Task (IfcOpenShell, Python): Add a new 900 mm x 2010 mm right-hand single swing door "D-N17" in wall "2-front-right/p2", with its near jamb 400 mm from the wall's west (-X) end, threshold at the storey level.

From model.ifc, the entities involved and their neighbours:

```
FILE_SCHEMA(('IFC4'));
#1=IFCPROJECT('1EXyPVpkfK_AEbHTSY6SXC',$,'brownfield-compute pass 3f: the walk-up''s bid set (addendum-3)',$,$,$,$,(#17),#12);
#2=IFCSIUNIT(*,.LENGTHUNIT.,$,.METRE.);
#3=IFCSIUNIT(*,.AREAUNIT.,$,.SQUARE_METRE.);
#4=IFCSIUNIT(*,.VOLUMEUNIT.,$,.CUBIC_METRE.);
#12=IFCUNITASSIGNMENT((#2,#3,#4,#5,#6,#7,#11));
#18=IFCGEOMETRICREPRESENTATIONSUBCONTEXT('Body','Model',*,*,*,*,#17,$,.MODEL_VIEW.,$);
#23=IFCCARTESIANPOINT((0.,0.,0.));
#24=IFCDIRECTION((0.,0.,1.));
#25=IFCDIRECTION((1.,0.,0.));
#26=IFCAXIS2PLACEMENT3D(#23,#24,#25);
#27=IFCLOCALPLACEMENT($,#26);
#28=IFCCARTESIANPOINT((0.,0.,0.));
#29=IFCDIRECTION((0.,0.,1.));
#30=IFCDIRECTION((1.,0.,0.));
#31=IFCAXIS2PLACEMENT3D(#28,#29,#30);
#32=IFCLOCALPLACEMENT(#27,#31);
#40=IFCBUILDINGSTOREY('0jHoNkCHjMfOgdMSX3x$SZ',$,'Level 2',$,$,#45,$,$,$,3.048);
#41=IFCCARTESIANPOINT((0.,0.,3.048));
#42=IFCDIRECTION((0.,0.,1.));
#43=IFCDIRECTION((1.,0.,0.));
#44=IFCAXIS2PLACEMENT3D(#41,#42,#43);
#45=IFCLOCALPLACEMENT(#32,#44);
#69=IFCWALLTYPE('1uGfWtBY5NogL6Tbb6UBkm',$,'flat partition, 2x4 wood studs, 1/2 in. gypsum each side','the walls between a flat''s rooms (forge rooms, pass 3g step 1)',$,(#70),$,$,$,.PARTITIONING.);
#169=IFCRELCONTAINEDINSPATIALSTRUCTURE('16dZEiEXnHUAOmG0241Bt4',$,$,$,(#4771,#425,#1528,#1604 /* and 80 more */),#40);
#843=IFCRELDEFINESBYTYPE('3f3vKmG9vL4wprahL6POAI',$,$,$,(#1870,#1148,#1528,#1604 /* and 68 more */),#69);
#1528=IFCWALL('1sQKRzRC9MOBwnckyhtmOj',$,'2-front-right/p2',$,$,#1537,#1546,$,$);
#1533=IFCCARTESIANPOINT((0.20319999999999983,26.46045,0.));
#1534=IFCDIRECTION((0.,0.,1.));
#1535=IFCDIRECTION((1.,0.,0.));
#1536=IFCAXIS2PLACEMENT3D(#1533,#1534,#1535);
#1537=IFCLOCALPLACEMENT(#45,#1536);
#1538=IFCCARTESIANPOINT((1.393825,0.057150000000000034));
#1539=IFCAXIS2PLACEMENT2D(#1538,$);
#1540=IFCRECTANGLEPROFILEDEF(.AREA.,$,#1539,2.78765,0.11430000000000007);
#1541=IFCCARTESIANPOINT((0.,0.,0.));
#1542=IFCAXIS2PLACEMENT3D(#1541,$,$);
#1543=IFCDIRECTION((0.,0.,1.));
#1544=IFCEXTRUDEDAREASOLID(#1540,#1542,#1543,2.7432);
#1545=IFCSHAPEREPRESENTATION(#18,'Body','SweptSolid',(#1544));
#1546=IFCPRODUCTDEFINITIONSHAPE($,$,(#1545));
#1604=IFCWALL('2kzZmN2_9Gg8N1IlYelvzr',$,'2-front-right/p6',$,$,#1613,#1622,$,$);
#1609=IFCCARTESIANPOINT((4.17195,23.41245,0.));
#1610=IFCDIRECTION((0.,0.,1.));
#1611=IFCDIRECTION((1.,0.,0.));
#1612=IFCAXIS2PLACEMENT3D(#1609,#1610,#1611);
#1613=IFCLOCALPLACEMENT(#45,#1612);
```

```python
import numpy as np
import ifcopenshell
import ifcopenshell.api.feature
import ifcopenshell.api.geometry
import ifcopenshell.api.root
import ifcopenshell.api.spatial
import ifcopenshell.geom
import ifcopenshell.util.element
import ifcopenshell.util.placement
import ifcopenshell.util.representation
import ifcopenshell.util.shape
import ifcopenshell.util.unit

model = ifcopenshell.open("model.ifc")
unit_scale = ifcopenshell.util.unit.calculate_unit_scale(model)
settings = ifcopenshell.geom.settings()


def volume(element):
    """Net volume in cubic metres, openings subtracted."""
    shape = ifcopenshell.geom.create_shape(settings, element)
    return ifcopenshell.util.shape.get_volume(shape.geometry)


wall = model.by_guid("1sQKRzRC9MOBwnckyhtmOj")
storey = ifcopenshell.util.element.get_container(wall, ifc_class="IfcBuildingStorey")
context = ifcopenshell.util.representation.get_context(model, "Model", "Body", "MODEL_VIEW")
before = volume(wall)

width, height, from_end, sill = 0.9, 2.01, 0.4, 0.0  # metres

# The wall runs along its own X axis, and the end named is its -X end.
wall_shape = ifcopenshell.geom.create_shape(settings, wall)
x, y, z = ifcopenshell.util.shape.get_vertices(wall_shape.geometry).T
start = x.min() + from_end
face, thickness = float(y.min()), float(y.max() - y.min())
wall_matrix = ifcopenshell.util.placement.get_local_placement(wall.ObjectPlacement)
level = ifcopenshell.util.placement.get_local_placement(storey.ObjectPlacement)[2, 3]


def in_wall(x, y):
    """Placement at x, y metres in the wall's axes, at sill height."""
    matrix = wall_matrix.copy()
    matrix[:, 3] = wall_matrix @ np.array([x / unit_scale, y / unit_scale, 0.0, 1.0])
    matrix[2, 3] = level + sill / unit_scale
    return matrix


# Opening: a box that overshoots both wall faces by 50 mm.
opening = ifcopenshell.api.root.create_entity(model, ifc_class="IfcOpeningElement", predefined_type="OPENING")
box = ifcopenshell.api.geometry.add_wall_representation(
    model, context=context, length=width, height=height, thickness=thickness + 0.1
)
ifcopenshell.api.geometry.assign_representation(model, product=opening, representation=box)
ifcopenshell.api.geometry.edit_object_placement(model, product=opening, matrix=in_wall(start, face - 0.05), is_si=False)
ifcopenshell.api.feature.add_feature(model, feature=opening, element=wall)

door = ifcopenshell.api.root.create_entity(model, ifc_class="IfcDoor", name="D-N17", predefined_type="DOOR")
door.OverallWidth, door.OverallHeight = width / unit_scale, height / unit_scale
door.OperationType = "SINGLE_SWING_RIGHT"
body = ifcopenshell.api.geometry.add_door_representation(
    model,
    context=context,
    overall_width=door.OverallWidth,
    overall_height=door.OverallHeight,
    operation_type="SINGLE_SWING_RIGHT",
    lining_properties={"LiningDepth": thickness / unit_scale, "ThresholdDepth": thickness / unit_scale},
)
ifcopenshell.api.geometry.assign_representation(model, product=door, representation=body)
ifcopenshell.api.spatial.assign_container(model, products=[door], relating_structure=storey)
ifcopenshell.api.feature.add_filling(model, opening=opening, element=door)

# The lining spans the wall, so the door starts at the wall face.
ifcopenshell.api.geometry.edit_object_placement(model, product=door, matrix=in_wall(start, face), is_si=False)

after = volume(wall)

print(f"wall volume {before:.3f} -> {after:.3f} m3")

model.write("model_edited.ifc")
```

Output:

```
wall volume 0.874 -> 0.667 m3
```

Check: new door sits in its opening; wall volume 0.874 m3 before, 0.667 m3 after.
